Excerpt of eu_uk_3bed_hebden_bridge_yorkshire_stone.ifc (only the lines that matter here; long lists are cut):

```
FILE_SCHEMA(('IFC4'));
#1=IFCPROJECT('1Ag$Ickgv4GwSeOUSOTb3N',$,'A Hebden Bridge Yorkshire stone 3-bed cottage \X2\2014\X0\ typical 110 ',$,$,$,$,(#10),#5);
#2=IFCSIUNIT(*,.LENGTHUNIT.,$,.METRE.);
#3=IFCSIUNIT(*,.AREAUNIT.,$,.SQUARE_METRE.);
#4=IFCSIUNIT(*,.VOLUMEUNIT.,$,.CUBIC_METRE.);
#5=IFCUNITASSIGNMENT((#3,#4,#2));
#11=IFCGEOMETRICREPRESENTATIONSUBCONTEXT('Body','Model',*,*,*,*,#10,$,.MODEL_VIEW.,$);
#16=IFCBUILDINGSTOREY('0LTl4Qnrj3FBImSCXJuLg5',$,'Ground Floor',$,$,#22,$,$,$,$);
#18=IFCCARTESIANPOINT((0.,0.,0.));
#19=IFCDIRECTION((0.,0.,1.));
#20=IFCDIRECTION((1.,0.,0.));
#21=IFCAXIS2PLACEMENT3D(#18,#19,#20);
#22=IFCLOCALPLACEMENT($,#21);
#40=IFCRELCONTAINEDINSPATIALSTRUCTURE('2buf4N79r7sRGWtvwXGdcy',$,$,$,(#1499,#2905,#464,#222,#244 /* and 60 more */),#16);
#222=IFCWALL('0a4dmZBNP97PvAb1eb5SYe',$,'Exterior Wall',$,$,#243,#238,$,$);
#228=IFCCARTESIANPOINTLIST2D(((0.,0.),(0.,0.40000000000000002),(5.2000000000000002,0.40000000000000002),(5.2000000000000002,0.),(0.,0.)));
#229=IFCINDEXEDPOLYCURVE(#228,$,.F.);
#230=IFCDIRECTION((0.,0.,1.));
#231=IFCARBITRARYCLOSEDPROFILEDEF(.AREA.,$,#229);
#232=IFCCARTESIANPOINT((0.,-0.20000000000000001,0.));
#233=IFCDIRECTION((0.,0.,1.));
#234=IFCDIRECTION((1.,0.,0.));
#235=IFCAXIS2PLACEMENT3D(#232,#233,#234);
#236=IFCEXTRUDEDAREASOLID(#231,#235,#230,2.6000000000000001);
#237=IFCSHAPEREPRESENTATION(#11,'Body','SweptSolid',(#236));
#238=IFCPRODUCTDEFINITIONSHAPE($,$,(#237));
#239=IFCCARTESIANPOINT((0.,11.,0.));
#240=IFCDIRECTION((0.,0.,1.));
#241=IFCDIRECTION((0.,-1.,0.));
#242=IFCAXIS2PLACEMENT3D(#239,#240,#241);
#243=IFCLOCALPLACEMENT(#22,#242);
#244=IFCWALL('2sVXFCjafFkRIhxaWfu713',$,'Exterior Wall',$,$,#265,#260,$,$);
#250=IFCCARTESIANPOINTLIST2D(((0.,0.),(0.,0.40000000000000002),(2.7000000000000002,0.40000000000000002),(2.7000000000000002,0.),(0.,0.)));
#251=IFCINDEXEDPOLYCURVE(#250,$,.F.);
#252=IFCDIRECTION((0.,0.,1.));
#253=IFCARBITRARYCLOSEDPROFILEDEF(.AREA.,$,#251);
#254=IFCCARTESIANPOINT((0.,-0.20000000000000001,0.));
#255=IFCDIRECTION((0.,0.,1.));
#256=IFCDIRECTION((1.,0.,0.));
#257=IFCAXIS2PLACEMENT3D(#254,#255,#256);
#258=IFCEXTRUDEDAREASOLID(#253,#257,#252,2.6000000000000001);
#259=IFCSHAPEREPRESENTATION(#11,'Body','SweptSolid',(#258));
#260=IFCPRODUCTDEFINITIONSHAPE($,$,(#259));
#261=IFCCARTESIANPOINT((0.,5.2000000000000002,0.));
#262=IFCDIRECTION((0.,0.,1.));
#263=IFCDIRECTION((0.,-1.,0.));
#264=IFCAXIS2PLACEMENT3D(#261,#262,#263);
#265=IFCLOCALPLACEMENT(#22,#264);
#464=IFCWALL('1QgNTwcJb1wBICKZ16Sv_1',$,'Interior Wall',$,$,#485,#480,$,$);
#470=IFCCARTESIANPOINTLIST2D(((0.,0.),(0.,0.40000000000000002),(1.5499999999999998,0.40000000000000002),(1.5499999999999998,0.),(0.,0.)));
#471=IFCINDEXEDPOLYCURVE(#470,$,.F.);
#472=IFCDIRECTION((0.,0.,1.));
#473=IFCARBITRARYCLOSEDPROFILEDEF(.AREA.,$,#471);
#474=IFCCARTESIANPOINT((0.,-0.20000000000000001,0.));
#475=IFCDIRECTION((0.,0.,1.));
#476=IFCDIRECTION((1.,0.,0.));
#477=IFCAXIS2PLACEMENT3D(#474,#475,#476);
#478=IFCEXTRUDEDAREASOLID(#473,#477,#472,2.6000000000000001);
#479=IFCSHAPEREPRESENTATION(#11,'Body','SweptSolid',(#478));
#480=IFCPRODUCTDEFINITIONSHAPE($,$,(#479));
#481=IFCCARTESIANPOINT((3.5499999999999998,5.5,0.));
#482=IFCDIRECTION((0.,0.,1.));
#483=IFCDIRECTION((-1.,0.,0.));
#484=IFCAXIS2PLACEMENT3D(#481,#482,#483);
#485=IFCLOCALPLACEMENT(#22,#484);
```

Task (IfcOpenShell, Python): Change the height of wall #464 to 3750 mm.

```python
import ifcopenshell
import ifcopenshell.geom
import ifcopenshell.util.representation
import ifcopenshell.util.shape

model = ifcopenshell.open("eu_uk_3bed_hebden_bridge_yorkshire_stone.ifc")
settings = ifcopenshell.geom.settings()


def volume(element):
    """Net volume in cubic metres, openings subtracted."""
    shape = ifcopenshell.geom.create_shape(settings, element)
    return ifcopenshell.util.shape.get_volume(shape.geometry)


wall = model.by_guid("1QgNTwcJb1wBICKZ16Sv_1")
before = volume(wall)

body = ifcopenshell.util.representation.get_representation(wall, "Model", "Body")
solid = body.Items[0]
old_height = solid.Depth
solid.Depth = 3.75
after = volume(wall)

print(f"height {old_height:g} -> {solid.Depth:g}, volume {before:.3f} -> {after:.3f} m3")

model.write("eu_uk_3bed_hebden_bridge_yorkshire_stone_edited.ifc")
```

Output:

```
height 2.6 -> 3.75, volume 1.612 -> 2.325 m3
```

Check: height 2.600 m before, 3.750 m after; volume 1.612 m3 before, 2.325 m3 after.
